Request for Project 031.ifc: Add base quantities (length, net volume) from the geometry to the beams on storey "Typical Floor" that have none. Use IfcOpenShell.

First a look at what the model holds.

```python
import ifcopenshell
import ifcopenshell.util.element
import ifcopenshell.util.unit

model = ifcopenshell.open("Project 031.ifc")
print(model.schema)
for unit_type in ("LENGTHUNIT", "AREAUNIT", "VOLUMEUNIT"):
    print(unit_type, ifcopenshell.util.unit.calculate_unit_scale(model, unit_type))
storey = next(s for s in model.by_type("IfcBuildingStorey") if s.Name == "Typical Floor")
beams = [e for e in ifcopenshell.util.element.get_decomposition(storey) if e.is_a("IfcBeam")]
for e in sorted(beams, key=lambda e: e.id()):
    print(e.id(), e.is_a(), e.Name, list(ifcopenshell.util.element.get_psets(e, qtos_only=True)), sep=" | ")
```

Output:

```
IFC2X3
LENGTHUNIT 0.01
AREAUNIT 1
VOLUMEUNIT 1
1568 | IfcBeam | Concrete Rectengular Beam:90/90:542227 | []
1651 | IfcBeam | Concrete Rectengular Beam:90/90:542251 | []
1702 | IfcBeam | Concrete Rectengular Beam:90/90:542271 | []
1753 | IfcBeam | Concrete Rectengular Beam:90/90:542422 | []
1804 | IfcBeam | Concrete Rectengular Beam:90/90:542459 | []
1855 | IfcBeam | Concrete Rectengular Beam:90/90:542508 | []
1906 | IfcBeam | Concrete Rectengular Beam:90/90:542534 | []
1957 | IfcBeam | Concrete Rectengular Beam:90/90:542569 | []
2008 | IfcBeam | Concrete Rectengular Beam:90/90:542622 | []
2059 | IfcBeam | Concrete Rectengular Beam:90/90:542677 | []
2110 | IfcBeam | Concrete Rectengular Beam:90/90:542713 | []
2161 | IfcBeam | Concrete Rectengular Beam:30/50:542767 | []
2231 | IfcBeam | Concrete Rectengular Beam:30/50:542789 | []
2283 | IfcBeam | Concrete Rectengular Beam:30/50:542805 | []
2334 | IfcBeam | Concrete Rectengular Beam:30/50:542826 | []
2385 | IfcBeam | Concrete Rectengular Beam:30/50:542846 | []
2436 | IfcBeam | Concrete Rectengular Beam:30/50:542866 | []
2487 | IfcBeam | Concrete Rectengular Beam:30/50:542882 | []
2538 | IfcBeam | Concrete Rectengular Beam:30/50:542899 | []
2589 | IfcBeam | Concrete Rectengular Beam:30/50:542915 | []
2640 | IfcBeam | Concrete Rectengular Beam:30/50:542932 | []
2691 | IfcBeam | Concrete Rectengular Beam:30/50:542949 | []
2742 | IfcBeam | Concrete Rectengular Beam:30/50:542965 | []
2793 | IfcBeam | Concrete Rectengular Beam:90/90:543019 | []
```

```python
import ifcopenshell
import ifcopenshell.api.pset
import ifcopenshell.geom
import ifcopenshell.util.element
import ifcopenshell.util.shape
import ifcopenshell.util.unit

model = ifcopenshell.open("Project 031.ifc")
unit_scale = ifcopenshell.util.unit.calculate_unit_scale(model)
volume_scale = ifcopenshell.util.unit.calculate_unit_scale(model, "VOLUMEUNIT")
settings = ifcopenshell.geom.settings()

storey = next(s for s in model.by_type("IfcBuildingStorey") if s.Name == "Typical Floor")
beams = [e for e in ifcopenshell.util.element.get_decomposition(storey) if e.is_a("IfcBeam")]

for e in sorted(beams, key=lambda e: e.id()):
    if ifcopenshell.util.element.get_psets(e, qtos_only=True, should_inherit=False):
        continue
    # Geometry comes back in metres, in the element's own axes.
    shape = ifcopenshell.geom.create_shape(settings, e)
    values = {
        "Length": ifcopenshell.util.shape.get_max_xyz(shape.geometry) / unit_scale,
        "NetVolume": ifcopenshell.util.shape.get_volume(shape.geometry) / volume_scale,
    }
    qto = ifcopenshell.api.pset.add_qto(model, product=e, name="BaseQuantities")
    ifcopenshell.api.pset.edit_qto(model, qto=qto, properties=values)
    print(e.id(), {k: round(v, 3) for k, v in values.items()})

model.write("Project 031_v2.ifc")
```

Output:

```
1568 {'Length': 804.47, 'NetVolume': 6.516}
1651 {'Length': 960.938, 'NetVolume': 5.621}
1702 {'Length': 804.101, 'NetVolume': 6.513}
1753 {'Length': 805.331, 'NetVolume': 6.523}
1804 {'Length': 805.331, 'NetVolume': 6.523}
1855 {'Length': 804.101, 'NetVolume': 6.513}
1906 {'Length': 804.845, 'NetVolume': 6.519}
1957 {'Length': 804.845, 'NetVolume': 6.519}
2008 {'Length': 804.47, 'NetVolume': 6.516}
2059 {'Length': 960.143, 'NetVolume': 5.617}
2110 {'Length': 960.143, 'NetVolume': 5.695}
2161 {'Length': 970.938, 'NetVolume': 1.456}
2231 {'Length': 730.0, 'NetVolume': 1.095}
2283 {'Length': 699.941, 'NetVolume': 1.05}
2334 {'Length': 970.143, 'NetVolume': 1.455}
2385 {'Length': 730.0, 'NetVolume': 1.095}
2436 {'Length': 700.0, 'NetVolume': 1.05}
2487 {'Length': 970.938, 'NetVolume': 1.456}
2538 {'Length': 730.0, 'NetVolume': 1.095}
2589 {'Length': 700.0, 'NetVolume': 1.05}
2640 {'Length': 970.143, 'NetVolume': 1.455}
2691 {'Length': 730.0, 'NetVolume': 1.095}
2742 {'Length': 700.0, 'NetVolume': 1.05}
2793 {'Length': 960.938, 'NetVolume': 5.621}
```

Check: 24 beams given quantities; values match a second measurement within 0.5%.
